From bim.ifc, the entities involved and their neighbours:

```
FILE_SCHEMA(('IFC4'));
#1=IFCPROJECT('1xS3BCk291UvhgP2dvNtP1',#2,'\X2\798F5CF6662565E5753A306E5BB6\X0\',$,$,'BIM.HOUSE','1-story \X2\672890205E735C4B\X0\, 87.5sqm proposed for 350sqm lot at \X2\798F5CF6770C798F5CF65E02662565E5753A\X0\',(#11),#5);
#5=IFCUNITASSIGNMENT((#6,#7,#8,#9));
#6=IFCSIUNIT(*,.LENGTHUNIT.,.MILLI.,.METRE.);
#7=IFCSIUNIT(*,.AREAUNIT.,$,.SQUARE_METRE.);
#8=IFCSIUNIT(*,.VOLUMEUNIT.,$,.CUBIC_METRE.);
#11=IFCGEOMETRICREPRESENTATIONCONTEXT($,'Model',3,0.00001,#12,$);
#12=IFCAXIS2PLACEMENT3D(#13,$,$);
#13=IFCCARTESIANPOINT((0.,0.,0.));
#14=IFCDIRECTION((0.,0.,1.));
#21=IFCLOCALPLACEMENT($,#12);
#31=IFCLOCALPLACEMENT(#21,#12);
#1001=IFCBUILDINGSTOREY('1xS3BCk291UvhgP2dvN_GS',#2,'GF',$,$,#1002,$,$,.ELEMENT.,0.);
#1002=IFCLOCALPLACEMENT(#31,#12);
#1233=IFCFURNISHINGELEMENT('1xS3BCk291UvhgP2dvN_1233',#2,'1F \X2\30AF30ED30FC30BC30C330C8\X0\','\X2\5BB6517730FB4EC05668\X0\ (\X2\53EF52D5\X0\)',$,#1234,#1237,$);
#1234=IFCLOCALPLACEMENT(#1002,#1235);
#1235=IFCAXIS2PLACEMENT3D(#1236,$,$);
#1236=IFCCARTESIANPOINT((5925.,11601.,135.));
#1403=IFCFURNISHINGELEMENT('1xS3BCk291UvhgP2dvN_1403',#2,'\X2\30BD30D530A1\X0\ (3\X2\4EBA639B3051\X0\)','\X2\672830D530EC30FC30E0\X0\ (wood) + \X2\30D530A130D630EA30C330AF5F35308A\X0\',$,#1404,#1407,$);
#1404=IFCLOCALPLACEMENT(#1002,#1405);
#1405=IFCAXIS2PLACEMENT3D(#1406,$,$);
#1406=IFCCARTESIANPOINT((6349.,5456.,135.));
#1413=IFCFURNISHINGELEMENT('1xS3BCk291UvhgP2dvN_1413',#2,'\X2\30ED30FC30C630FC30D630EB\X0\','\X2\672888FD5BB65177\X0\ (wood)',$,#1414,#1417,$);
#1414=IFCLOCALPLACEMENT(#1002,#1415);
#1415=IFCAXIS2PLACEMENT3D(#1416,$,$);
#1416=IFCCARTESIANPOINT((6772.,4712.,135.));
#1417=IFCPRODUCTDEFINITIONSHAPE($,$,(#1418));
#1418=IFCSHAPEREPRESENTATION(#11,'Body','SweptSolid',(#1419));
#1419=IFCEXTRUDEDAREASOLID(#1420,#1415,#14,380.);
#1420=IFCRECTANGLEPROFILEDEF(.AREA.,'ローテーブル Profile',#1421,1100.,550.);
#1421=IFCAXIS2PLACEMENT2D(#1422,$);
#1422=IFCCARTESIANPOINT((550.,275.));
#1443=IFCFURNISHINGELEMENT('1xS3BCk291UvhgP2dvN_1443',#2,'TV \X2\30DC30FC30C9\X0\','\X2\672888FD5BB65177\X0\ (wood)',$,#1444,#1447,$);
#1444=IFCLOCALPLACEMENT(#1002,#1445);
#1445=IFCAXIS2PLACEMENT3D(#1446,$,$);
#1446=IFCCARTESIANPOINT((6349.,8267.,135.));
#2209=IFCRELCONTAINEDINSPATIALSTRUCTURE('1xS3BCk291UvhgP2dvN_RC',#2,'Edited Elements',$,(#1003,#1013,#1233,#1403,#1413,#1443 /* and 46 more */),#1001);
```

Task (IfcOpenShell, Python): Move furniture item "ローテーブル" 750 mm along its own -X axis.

```python
import ifcopenshell
import ifcopenshell.api.geometry
import ifcopenshell.util.placement
import ifcopenshell.util.unit

model = ifcopenshell.open("bim.ifc")
unit_scale = ifcopenshell.util.unit.calculate_unit_scale(model)

item = model.by_guid("1xS3BCk291UvhgP2dvN_1413")
matrix = ifcopenshell.util.placement.get_local_placement(item.ObjectPlacement)
matrix[:3, 3] -= matrix[:3, 0] * 0.75 / unit_scale
ifcopenshell.api.geometry.edit_object_placement(model, product=item, matrix=matrix, is_si=False)

print(ifcopenshell.util.placement.get_local_placement(item.ObjectPlacement).round(3) + 0.0)

model.write("bim-out.ifc")
```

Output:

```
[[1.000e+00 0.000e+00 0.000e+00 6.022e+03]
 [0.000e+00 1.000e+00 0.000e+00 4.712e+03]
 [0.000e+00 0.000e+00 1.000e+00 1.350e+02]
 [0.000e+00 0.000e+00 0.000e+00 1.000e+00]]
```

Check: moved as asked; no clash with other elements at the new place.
